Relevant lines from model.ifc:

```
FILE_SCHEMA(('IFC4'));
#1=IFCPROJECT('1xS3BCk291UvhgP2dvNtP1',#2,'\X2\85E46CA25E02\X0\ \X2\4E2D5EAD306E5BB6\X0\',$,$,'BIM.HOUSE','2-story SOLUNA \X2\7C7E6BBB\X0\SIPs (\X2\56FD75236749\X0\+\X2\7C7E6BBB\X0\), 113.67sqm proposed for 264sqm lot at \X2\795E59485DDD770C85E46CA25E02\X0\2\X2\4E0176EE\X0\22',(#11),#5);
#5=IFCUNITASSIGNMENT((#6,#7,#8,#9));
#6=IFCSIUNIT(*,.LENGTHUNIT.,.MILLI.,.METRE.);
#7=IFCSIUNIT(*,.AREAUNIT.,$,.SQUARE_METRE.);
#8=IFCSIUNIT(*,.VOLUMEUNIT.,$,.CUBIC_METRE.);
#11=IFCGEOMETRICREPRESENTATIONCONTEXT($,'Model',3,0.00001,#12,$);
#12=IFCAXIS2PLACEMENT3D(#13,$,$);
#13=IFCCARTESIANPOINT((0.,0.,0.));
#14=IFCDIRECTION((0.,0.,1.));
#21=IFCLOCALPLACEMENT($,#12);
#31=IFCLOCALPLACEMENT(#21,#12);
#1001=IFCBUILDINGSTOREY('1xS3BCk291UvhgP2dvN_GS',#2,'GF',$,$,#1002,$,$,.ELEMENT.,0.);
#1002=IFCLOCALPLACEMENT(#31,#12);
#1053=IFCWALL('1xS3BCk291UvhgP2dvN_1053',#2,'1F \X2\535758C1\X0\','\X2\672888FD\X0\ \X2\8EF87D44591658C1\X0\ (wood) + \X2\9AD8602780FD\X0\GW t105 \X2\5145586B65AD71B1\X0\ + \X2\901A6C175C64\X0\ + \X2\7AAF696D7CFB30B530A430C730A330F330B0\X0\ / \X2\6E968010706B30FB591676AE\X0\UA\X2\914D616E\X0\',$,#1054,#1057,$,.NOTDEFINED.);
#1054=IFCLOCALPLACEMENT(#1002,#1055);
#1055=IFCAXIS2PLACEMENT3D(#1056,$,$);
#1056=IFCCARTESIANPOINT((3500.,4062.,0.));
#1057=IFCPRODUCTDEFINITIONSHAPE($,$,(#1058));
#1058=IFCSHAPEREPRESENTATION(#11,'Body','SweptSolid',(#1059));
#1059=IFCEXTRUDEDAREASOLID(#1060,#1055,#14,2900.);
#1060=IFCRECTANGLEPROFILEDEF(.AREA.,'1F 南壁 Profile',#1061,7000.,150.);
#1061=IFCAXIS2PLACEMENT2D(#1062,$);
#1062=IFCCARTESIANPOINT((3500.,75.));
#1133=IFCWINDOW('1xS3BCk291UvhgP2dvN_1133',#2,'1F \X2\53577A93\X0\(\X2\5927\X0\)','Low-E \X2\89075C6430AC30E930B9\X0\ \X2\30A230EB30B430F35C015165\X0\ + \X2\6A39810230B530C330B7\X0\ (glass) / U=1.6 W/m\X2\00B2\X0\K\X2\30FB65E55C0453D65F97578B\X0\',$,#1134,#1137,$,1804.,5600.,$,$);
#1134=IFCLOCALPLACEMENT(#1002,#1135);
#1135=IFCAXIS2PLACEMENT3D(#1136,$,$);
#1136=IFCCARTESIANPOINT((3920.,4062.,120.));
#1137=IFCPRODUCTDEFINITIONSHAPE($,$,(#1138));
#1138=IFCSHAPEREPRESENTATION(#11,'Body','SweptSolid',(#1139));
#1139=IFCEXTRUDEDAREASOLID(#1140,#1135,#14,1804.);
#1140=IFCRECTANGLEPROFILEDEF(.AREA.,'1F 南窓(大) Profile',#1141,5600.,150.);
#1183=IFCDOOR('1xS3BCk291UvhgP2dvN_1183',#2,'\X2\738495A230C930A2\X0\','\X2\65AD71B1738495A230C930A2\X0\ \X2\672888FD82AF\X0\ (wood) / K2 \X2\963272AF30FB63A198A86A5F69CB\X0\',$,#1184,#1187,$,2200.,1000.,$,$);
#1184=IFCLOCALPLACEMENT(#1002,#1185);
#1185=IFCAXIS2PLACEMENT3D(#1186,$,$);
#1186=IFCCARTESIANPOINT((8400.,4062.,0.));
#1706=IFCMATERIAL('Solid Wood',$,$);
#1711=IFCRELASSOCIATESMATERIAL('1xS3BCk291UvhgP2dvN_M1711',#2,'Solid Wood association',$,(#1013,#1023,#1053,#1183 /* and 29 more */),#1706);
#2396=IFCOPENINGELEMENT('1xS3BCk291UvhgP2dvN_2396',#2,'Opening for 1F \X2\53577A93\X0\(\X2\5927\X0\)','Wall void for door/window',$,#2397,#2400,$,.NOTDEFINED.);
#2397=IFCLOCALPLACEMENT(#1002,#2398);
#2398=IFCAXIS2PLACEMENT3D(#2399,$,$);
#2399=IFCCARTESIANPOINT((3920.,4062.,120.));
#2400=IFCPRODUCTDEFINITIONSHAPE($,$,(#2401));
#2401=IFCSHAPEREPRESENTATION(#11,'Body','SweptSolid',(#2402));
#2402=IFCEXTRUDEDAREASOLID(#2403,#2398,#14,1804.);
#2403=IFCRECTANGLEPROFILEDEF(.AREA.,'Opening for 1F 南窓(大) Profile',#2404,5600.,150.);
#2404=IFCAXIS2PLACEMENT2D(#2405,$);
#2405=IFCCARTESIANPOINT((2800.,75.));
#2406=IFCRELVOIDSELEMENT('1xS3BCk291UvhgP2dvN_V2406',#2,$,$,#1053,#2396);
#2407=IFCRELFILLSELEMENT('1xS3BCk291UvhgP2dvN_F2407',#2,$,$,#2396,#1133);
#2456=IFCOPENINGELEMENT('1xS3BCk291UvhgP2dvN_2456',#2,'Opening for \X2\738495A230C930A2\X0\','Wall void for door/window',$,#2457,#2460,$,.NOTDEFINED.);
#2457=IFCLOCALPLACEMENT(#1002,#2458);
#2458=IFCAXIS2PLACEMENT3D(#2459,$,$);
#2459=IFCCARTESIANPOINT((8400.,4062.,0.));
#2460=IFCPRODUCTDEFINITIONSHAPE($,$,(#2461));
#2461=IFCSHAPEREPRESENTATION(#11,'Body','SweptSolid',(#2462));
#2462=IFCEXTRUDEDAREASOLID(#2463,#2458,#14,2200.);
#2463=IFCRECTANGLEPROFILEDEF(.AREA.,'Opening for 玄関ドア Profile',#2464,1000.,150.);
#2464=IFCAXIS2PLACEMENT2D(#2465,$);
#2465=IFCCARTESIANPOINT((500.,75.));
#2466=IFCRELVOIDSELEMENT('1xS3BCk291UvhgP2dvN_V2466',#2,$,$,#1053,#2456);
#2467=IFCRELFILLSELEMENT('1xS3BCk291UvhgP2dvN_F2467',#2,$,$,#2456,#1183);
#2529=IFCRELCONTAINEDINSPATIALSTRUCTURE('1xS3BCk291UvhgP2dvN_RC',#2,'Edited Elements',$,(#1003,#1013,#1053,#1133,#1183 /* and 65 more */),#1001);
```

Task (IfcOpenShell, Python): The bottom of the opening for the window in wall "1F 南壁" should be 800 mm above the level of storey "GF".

```python
import numpy as np
import ifcopenshell
import ifcopenshell.api.geometry
import ifcopenshell.geom
import ifcopenshell.util.element
import ifcopenshell.util.placement
import ifcopenshell.util.shape
import ifcopenshell.util.unit

model = ifcopenshell.open("model.ifc")
unit_scale = ifcopenshell.util.unit.calculate_unit_scale(model)

window = model.by_id(1133)
opening = window.FillsVoids[0].RelatingOpeningElement
storey = ifcopenshell.util.element.get_container(window, ifc_class="IfcBuildingStorey")
level = ifcopenshell.util.placement.get_local_placement(storey.ObjectPlacement)[2, 3]

# The opening's origin need not be at the sill, so measure its lowest point.
shape = ifcopenshell.geom.create_shape(ifcopenshell.geom.settings(), opening)
bottom = ifcopenshell.util.shape.get_shape_bottom_elevation(shape, shape.geometry) / unit_scale
dz = level + 0.8 / unit_scale - bottom

shift = np.array([0.0, 0.0, dz])
# The window is not placed relative to its opening, so move both.
for product in (opening, window):
    matrix = ifcopenshell.util.placement.get_local_placement(product.ObjectPlacement)
    matrix[:3, 3] += shift
    ifcopenshell.api.geometry.edit_object_placement(model, product=product, matrix=matrix, is_si=False)

print(f"moved by {dz * unit_scale:+.3f} m")

model.write("model_edited.ifc")
```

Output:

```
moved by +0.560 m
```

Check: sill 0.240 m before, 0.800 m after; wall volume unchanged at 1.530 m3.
